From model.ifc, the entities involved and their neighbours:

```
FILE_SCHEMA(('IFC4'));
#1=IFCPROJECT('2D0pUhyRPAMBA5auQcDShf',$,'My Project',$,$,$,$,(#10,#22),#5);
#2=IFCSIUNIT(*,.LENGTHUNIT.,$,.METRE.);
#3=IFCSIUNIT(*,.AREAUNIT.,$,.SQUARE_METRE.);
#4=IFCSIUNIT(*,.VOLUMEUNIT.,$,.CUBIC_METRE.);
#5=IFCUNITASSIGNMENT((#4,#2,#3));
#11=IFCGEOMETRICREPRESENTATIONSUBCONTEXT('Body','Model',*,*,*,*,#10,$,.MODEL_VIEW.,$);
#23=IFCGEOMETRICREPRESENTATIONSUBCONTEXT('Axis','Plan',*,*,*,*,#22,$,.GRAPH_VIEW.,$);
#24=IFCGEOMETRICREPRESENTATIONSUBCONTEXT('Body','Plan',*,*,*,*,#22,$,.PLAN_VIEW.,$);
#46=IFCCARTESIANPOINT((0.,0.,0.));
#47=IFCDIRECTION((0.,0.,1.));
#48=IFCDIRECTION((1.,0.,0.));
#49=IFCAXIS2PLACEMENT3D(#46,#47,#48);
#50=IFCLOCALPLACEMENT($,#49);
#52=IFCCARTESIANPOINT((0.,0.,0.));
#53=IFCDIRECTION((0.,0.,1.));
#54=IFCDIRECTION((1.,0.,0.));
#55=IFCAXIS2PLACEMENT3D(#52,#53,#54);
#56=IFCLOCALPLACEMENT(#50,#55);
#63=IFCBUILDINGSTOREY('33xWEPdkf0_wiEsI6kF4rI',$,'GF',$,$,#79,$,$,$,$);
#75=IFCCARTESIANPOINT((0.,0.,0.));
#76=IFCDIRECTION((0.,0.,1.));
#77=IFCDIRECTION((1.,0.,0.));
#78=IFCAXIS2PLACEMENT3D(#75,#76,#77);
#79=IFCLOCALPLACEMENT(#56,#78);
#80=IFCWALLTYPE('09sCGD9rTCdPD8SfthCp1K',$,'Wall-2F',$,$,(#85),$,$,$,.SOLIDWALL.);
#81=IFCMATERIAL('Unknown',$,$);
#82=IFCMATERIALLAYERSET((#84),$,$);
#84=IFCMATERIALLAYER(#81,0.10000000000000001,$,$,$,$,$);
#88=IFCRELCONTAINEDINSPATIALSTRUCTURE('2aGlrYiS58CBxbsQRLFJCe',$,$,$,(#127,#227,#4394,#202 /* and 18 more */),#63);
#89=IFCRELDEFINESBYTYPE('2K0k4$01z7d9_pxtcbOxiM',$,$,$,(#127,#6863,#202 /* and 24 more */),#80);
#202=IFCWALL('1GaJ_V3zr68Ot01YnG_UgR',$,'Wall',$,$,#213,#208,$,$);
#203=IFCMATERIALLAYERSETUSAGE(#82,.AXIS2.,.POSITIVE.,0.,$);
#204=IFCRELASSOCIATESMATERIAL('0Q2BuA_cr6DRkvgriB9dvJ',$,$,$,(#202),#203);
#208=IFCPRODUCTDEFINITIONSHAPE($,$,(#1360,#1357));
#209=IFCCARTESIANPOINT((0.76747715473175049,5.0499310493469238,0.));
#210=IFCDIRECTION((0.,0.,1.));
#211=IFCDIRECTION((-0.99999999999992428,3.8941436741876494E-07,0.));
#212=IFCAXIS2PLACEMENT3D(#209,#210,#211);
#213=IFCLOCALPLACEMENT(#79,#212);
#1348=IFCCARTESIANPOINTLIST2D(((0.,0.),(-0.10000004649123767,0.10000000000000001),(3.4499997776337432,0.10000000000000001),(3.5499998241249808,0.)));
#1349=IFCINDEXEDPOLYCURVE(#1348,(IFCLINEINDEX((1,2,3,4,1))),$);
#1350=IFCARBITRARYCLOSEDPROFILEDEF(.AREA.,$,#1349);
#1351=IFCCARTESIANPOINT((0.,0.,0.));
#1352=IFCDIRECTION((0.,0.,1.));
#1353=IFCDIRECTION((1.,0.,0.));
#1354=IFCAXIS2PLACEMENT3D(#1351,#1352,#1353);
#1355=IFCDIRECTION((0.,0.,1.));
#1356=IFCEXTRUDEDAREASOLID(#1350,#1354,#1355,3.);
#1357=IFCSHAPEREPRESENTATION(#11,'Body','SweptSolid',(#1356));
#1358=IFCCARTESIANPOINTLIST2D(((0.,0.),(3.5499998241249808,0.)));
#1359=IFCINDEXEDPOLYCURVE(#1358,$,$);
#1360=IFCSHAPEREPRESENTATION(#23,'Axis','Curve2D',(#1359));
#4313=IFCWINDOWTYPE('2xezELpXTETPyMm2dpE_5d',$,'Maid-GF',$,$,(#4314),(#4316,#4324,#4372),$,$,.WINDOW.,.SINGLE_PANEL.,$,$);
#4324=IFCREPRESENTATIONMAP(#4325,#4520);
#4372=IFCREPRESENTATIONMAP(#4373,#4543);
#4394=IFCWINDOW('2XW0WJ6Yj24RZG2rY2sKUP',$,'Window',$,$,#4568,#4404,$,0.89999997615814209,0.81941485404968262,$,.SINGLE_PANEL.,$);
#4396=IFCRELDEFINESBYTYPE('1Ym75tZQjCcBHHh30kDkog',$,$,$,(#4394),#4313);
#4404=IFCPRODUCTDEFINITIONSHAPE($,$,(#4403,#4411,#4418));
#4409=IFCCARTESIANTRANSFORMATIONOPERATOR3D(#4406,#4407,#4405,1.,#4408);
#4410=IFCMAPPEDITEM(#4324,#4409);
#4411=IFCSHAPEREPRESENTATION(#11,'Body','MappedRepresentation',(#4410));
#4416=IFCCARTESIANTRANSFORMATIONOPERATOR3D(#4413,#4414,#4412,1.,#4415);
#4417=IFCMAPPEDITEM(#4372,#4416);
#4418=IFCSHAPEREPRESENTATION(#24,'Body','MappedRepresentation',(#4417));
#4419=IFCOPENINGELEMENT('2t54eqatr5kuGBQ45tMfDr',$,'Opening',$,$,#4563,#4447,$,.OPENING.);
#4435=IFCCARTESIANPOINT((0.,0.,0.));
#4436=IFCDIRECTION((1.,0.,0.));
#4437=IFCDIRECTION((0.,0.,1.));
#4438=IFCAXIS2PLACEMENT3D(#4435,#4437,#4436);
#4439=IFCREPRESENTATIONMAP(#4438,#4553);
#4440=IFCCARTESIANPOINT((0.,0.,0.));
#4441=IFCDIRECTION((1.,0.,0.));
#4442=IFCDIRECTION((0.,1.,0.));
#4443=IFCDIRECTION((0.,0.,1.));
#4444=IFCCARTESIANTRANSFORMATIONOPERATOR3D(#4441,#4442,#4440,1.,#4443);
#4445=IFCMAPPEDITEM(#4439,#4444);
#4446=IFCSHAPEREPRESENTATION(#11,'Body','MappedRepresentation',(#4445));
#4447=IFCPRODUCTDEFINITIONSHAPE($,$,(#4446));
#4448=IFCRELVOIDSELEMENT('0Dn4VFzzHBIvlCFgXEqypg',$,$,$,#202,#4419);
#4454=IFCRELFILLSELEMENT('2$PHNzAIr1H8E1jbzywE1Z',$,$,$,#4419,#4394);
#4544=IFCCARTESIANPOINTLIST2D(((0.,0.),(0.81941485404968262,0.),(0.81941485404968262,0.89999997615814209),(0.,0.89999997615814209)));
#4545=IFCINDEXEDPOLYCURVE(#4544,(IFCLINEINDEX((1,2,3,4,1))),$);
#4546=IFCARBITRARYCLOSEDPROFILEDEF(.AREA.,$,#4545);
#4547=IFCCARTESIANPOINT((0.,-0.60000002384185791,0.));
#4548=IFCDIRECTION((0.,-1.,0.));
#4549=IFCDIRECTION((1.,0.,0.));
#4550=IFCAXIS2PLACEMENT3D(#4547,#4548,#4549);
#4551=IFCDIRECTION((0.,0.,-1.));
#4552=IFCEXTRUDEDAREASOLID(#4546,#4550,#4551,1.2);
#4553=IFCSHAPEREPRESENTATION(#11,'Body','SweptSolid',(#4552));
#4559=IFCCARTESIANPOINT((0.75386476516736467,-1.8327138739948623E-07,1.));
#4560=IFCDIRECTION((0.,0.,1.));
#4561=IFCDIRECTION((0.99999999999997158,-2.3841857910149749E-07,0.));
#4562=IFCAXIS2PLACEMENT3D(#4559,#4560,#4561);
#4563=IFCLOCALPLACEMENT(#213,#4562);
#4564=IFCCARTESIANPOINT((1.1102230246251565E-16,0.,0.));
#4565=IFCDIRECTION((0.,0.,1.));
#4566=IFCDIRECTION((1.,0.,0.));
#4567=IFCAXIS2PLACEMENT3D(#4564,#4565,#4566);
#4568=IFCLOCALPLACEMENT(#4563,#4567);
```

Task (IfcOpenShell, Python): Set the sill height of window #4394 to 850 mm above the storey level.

```python
import numpy as np
import ifcopenshell
import ifcopenshell.api.geometry
import ifcopenshell.geom
import ifcopenshell.util.element
import ifcopenshell.util.placement
import ifcopenshell.util.shape
import ifcopenshell.util.unit

model = ifcopenshell.open("model.ifc")
unit_scale = ifcopenshell.util.unit.calculate_unit_scale(model)

window = model.by_guid("2XW0WJ6Yj24RZG2rY2sKUP")
opening = window.FillsVoids[0].RelatingOpeningElement
storey = ifcopenshell.util.element.get_container(window, ifc_class="IfcBuildingStorey")
level = ifcopenshell.util.placement.get_local_placement(storey.ObjectPlacement)[2, 3]

# The opening's origin need not be at the sill, so measure its lowest point.
shape = ifcopenshell.geom.create_shape(ifcopenshell.geom.settings(), opening)
bottom = ifcopenshell.util.shape.get_shape_bottom_elevation(shape, shape.geometry) / unit_scale
dz = level + 0.85 / unit_scale - bottom

shift = np.array([0.0, 0.0, dz])
# The window is placed relative to its opening, so it follows when the opening moves.
matrix = ifcopenshell.util.placement.get_local_placement(opening.ObjectPlacement)
matrix[:3, 3] += shift
ifcopenshell.api.geometry.edit_object_placement(
    model, product=opening, matrix=matrix, is_si=False, should_transform_children=True
)

print(f"moved by {dz * unit_scale:+.3f} m")

model.write("model_rev.ifc")
```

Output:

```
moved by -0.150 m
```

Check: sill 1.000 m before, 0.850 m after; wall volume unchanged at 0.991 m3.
